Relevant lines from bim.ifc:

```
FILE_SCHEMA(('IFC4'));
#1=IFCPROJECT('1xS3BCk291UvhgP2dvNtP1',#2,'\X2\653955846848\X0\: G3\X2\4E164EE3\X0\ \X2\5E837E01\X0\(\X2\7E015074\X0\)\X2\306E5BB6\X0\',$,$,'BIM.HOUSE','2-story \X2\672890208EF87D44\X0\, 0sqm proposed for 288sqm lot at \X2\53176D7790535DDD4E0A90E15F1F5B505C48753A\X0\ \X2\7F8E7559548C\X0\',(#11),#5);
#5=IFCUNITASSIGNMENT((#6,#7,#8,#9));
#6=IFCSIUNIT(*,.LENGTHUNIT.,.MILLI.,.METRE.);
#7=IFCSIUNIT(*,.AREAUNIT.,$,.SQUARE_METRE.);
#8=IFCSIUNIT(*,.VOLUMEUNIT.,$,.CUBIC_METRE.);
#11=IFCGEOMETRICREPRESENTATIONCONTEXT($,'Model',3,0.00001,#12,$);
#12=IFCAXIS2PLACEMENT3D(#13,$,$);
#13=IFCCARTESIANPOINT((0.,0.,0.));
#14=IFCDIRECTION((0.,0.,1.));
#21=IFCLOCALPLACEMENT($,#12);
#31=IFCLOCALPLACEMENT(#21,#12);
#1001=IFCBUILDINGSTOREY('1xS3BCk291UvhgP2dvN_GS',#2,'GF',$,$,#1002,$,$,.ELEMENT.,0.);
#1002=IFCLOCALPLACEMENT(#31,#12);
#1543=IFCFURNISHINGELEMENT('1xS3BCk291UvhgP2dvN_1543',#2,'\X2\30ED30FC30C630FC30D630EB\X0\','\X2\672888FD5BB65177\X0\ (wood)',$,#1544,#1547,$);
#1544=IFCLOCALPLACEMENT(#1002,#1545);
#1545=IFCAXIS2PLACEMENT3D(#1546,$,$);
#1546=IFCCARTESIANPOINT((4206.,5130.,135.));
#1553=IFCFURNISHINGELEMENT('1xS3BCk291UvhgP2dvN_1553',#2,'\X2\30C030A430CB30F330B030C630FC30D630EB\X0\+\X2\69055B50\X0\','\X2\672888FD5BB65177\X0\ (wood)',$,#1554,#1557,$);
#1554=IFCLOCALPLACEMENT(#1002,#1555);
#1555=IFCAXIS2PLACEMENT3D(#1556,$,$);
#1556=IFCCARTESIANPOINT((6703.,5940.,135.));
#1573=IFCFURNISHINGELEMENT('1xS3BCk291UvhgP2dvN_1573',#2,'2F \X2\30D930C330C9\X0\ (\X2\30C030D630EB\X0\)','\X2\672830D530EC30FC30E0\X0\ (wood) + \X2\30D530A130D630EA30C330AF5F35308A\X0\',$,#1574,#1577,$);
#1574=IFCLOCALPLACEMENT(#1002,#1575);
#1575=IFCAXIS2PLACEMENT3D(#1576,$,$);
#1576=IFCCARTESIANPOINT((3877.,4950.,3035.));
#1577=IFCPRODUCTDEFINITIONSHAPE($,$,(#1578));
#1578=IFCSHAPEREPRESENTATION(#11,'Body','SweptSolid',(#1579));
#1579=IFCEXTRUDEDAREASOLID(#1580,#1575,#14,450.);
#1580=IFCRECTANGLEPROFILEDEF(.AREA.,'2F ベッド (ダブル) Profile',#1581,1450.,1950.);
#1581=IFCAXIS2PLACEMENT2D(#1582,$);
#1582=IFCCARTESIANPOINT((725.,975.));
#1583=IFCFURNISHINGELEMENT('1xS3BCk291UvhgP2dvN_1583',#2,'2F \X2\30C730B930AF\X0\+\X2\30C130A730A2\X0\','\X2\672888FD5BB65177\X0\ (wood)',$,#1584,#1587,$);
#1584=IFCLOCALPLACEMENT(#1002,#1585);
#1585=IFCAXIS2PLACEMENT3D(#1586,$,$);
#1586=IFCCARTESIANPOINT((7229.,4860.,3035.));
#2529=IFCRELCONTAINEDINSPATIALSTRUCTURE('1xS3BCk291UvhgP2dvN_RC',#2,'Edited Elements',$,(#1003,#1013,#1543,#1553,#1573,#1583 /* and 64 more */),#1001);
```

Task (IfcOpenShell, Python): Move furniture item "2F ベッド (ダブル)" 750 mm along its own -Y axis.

```python
import ifcopenshell
import ifcopenshell.api.geometry
import ifcopenshell.util.placement
import ifcopenshell.util.unit

model = ifcopenshell.open("bim.ifc")
unit_scale = ifcopenshell.util.unit.calculate_unit_scale(model)

item = model.by_guid("1xS3BCk291UvhgP2dvN_1573")
matrix = ifcopenshell.util.placement.get_local_placement(item.ObjectPlacement)
matrix[:3, 3] -= matrix[:3, 1] * 0.75 / unit_scale
ifcopenshell.api.geometry.edit_object_placement(model, product=item, matrix=matrix, is_si=False)

print(ifcopenshell.util.placement.get_local_placement(item.ObjectPlacement).round(3) + 0.0)

model.write("bim_rev.ifc")
```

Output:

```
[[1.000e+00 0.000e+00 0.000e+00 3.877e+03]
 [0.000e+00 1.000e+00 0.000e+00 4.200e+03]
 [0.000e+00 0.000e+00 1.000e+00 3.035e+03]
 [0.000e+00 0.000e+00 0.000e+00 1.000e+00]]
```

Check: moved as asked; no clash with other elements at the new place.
